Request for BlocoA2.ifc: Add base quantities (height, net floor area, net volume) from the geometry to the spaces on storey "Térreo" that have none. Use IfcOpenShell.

First a look at what the model holds.

```python
import ifcopenshell
import ifcopenshell.util.element
import ifcopenshell.util.unit

model = ifcopenshell.open("BlocoA2.ifc")
print(model.schema)
for unit_type in ("LENGTHUNIT", "AREAUNIT", "VOLUMEUNIT"):
    print(unit_type, ifcopenshell.util.unit.calculate_unit_scale(model, unit_type))
storey = next(s for s in model.by_type("IfcBuildingStorey") if s.Name == "Térreo")
spaces = [e for e in ifcopenshell.util.element.get_decomposition(storey) if e.is_a("IfcSpace")]
for e in sorted(spaces, key=lambda e: e.id()):
    print(e.id(), e.is_a(), e.Name, list(ifcopenshell.util.element.get_psets(e, qtos_only=True)), sep=" | ")
```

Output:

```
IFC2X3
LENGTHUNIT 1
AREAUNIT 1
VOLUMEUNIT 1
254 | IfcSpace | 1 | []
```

```python
import ifcopenshell
import ifcopenshell.api.pset
import ifcopenshell.geom
import ifcopenshell.util.element
import ifcopenshell.util.shape
import ifcopenshell.util.unit

model = ifcopenshell.open("BlocoA2.ifc")
unit_scale = ifcopenshell.util.unit.calculate_unit_scale(model)
area_scale = ifcopenshell.util.unit.calculate_unit_scale(model, "AREAUNIT")
volume_scale = ifcopenshell.util.unit.calculate_unit_scale(model, "VOLUMEUNIT")
settings = ifcopenshell.geom.settings()

storey = next(s for s in model.by_type("IfcBuildingStorey") if s.Name == "Térreo")
spaces = [e for e in ifcopenshell.util.element.get_decomposition(storey) if e.is_a("IfcSpace")]

for e in sorted(spaces, key=lambda e: e.id()):
    if ifcopenshell.util.element.get_psets(e, qtos_only=True, should_inherit=False):
        continue
    # Geometry comes back in metres, in the element's own axes.
    shape = ifcopenshell.geom.create_shape(settings, e)
    values = {
        "Height": ifcopenshell.util.shape.get_z(shape.geometry) / unit_scale,
        "NetFloorArea": ifcopenshell.util.shape.get_footprint_area(shape.geometry) / area_scale,
        "NetVolume": ifcopenshell.util.shape.get_volume(shape.geometry) / volume_scale,
    }
    qto = ifcopenshell.api.pset.add_qto(model, product=e, name="BaseQuantities")
    ifcopenshell.api.pset.edit_qto(model, qto=qto, properties=values)
    print(e.id(), {k: round(v, 3) for k, v in values.items()})

model.write("BlocoA2-out.ifc")
```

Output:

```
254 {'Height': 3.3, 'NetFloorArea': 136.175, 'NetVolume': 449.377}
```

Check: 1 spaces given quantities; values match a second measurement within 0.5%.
